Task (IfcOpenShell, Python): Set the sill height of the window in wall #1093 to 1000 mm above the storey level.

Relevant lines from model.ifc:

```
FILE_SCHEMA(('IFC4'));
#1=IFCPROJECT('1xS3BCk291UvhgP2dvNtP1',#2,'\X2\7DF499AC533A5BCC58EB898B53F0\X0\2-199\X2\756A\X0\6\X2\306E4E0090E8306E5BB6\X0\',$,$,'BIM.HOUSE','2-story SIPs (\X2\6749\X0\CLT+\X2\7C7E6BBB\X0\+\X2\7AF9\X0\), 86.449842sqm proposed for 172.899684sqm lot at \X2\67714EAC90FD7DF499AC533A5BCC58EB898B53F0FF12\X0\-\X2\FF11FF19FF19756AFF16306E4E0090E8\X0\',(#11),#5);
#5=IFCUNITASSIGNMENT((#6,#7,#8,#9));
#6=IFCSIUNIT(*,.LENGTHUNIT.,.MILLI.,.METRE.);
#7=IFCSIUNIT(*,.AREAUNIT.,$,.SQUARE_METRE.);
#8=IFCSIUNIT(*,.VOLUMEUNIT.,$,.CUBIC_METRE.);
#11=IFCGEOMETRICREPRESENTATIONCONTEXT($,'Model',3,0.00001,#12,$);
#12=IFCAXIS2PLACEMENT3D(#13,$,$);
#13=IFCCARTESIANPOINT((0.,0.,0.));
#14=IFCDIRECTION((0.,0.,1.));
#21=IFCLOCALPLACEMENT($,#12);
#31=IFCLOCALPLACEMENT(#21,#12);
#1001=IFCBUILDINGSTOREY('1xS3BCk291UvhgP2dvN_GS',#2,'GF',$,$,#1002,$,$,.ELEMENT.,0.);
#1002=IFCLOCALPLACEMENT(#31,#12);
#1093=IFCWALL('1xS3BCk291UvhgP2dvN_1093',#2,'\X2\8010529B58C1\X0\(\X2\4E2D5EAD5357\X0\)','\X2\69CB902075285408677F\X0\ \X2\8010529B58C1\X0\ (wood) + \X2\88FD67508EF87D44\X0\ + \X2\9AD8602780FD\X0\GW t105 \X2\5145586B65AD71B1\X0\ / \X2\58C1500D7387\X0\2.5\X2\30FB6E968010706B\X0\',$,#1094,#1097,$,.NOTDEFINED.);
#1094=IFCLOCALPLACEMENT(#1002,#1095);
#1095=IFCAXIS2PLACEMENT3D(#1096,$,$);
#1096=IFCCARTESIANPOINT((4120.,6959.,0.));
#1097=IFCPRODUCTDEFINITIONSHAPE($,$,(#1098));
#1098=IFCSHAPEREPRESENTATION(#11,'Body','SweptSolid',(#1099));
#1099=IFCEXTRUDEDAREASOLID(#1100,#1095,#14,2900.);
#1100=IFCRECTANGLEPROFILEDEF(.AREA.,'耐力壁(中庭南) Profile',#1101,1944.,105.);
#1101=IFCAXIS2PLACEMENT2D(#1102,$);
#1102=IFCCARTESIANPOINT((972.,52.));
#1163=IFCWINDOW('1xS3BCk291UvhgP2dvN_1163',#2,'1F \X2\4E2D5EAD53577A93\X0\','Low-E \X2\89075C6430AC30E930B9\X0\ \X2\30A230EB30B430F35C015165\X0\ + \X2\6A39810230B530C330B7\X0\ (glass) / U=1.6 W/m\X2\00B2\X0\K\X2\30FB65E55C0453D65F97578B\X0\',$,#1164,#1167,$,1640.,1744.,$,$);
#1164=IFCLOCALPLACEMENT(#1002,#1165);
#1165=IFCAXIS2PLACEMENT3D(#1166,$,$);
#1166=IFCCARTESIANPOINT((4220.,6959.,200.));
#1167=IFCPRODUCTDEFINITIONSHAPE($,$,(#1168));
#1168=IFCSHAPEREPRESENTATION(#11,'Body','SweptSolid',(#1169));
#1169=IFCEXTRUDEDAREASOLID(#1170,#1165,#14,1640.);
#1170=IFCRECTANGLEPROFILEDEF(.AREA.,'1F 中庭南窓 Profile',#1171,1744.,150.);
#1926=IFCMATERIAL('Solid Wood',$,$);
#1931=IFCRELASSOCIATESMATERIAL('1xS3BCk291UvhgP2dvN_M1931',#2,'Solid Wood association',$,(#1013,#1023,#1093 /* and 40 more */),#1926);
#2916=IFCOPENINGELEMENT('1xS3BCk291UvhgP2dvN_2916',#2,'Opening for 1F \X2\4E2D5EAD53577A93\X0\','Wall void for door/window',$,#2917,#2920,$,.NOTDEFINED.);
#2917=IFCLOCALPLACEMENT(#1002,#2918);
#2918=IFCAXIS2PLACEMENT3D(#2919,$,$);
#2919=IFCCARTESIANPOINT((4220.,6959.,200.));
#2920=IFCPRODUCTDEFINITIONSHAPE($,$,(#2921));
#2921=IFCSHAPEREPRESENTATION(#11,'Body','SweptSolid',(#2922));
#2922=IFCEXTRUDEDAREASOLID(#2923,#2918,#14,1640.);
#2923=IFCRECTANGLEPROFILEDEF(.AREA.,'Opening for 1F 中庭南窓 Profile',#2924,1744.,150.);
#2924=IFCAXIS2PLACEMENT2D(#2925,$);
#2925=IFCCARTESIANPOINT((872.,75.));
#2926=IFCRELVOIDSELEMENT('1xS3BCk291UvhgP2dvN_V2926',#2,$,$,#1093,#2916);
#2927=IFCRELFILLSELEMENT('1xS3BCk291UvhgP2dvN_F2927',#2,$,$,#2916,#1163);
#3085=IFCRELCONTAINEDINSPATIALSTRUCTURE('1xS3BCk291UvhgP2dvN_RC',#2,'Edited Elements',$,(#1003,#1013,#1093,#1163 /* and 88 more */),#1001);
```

```python
import numpy as np
import ifcopenshell
import ifcopenshell.api.geometry
import ifcopenshell.geom
import ifcopenshell.util.element
import ifcopenshell.util.placement
import ifcopenshell.util.shape
import ifcopenshell.util.unit

model = ifcopenshell.open("model.ifc")
unit_scale = ifcopenshell.util.unit.calculate_unit_scale(model)

window = model.by_id(1163)
opening = window.FillsVoids[0].RelatingOpeningElement
storey = ifcopenshell.util.element.get_container(window, ifc_class="IfcBuildingStorey")
level = ifcopenshell.util.placement.get_local_placement(storey.ObjectPlacement)[2, 3]

# The opening's origin need not be at the sill, so measure its lowest point.
shape = ifcopenshell.geom.create_shape(ifcopenshell.geom.settings(), opening)
bottom = ifcopenshell.util.shape.get_shape_bottom_elevation(shape, shape.geometry) / unit_scale
dz = level + 1 / unit_scale - bottom

shift = np.array([0.0, 0.0, dz])
# The window is not placed relative to its opening, so move both.
for product in (opening, window):
    matrix = ifcopenshell.util.placement.get_local_placement(product.ObjectPlacement)
    matrix[:3, 3] += shift
    ifcopenshell.api.geometry.edit_object_placement(model, product=product, matrix=matrix, is_si=False)

print(f"moved by {dz * unit_scale:+.3f} m")

model.write("model_rev.ifc")
```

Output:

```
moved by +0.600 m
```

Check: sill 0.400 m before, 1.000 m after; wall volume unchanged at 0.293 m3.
